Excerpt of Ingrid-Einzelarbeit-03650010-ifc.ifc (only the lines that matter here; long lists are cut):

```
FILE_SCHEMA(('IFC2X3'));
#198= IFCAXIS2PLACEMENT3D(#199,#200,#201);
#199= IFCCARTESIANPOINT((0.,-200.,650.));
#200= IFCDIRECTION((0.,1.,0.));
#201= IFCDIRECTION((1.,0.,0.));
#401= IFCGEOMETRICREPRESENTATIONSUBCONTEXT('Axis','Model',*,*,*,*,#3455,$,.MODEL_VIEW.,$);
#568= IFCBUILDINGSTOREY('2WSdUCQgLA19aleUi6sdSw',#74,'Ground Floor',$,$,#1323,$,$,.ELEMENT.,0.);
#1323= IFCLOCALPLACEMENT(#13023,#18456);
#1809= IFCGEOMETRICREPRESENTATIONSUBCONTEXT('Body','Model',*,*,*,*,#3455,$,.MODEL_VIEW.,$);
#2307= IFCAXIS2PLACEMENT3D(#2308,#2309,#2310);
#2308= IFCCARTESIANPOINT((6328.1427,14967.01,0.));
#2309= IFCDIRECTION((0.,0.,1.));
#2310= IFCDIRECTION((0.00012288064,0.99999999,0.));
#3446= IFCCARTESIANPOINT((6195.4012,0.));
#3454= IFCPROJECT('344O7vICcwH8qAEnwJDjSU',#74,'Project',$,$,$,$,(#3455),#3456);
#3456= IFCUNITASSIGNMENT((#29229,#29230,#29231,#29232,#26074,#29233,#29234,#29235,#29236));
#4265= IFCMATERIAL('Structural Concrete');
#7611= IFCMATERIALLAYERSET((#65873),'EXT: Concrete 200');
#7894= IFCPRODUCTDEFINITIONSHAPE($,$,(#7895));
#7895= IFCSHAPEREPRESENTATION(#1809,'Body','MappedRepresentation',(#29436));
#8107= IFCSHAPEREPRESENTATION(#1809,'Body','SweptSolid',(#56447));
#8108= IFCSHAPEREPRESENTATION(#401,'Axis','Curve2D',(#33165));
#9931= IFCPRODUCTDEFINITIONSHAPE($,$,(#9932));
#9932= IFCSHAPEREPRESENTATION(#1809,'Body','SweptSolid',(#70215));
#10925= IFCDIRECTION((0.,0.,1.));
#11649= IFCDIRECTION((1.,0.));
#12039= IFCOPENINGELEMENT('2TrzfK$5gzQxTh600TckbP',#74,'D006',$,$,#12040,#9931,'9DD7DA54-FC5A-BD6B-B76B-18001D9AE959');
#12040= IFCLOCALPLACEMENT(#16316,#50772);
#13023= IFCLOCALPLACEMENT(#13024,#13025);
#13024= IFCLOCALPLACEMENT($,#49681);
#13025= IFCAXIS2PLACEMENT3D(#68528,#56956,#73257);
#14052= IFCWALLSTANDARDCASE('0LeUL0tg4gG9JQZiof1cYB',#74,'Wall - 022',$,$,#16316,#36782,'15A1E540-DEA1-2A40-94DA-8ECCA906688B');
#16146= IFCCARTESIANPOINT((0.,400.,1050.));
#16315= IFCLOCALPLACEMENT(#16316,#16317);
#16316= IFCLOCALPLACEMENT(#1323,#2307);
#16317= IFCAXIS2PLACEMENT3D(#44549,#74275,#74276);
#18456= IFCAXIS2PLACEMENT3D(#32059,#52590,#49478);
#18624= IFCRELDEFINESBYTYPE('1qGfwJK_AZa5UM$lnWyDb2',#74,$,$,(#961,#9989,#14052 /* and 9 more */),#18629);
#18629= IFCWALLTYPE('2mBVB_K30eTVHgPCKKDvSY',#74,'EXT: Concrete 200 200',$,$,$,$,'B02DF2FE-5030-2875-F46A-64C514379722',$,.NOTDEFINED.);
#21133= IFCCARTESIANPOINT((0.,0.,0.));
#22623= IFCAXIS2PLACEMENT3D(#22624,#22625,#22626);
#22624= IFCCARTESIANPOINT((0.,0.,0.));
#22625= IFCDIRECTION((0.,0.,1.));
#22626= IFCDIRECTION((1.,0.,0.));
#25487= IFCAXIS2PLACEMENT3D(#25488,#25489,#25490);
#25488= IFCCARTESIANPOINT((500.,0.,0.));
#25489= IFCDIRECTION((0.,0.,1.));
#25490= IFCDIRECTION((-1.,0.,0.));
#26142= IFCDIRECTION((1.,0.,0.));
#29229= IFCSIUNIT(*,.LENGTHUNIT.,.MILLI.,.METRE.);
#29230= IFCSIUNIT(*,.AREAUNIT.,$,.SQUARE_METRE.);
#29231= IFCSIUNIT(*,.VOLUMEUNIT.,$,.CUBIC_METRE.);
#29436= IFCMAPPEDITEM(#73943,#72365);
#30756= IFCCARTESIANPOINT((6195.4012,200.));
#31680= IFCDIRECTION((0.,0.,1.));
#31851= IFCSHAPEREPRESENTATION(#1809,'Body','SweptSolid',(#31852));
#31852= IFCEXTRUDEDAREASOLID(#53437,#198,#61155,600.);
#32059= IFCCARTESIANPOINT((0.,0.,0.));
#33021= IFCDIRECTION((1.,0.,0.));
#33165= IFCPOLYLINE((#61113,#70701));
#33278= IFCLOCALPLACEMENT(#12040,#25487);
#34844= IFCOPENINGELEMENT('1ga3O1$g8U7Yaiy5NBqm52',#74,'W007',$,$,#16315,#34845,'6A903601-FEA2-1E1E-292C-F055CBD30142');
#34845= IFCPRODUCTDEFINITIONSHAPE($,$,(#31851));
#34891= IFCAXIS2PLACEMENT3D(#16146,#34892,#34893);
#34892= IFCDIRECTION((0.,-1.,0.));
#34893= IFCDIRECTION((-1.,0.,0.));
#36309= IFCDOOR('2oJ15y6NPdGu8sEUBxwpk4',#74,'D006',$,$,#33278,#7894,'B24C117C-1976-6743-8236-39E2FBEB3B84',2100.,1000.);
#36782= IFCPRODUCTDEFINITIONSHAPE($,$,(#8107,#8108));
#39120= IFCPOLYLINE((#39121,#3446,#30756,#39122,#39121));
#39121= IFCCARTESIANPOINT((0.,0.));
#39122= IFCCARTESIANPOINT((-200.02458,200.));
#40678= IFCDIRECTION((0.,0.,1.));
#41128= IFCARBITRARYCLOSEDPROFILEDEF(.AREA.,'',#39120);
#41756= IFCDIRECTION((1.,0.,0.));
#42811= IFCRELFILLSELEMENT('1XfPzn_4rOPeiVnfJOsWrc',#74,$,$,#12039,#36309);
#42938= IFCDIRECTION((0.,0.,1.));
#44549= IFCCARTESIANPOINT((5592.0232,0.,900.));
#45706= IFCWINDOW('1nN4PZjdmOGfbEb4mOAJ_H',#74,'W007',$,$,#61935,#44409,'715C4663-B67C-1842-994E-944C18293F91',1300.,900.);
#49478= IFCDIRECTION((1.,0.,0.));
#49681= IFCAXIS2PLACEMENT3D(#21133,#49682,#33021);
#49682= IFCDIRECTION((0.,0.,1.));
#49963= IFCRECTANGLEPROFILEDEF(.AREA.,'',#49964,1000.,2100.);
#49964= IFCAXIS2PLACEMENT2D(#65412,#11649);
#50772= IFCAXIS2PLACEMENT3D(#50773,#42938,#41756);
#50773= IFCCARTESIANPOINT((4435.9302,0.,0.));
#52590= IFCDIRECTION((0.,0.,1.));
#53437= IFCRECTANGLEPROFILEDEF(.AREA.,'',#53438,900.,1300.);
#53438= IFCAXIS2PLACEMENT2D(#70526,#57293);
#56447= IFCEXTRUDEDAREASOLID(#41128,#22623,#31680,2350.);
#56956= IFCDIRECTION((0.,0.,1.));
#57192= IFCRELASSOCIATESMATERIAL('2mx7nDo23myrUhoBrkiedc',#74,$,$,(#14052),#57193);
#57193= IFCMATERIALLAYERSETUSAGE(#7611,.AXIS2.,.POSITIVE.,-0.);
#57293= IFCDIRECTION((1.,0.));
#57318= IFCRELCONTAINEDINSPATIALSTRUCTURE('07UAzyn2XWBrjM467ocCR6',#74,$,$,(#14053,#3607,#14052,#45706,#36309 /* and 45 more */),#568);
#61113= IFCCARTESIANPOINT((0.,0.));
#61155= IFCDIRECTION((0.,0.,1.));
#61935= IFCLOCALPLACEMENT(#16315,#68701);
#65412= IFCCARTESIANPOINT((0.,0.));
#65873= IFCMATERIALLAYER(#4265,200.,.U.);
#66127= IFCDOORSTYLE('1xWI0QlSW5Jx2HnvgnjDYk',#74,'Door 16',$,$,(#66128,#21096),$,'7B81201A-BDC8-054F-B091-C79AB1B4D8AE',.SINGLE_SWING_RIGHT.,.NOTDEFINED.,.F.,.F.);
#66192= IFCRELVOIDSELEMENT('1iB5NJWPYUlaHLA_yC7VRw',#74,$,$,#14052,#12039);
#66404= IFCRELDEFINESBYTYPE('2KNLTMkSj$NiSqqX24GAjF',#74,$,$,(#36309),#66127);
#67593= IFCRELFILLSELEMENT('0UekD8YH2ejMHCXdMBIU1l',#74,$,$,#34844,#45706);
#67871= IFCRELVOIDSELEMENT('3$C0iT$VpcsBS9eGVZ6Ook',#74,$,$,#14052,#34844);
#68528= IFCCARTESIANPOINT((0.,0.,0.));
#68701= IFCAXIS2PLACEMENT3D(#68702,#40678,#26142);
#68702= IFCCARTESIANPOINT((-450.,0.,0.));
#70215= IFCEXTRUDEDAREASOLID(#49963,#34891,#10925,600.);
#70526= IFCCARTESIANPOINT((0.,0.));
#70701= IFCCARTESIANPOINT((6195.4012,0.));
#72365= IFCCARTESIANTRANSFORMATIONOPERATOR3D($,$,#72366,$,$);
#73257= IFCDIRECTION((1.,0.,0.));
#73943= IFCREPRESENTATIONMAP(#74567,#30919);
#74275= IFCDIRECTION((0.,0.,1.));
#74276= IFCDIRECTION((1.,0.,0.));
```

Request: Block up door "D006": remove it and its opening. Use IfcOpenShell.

```python
import ifcopenshell
import ifcopenshell.api.feature
import ifcopenshell.api.root
import ifcopenshell.geom
import ifcopenshell.util.shape

model = ifcopenshell.open("Ingrid-Einzelarbeit-03650010-ifc.ifc")
settings = ifcopenshell.geom.settings()


def volume(element):
    """Net volume in cubic metres, openings subtracted."""
    shape = ifcopenshell.geom.create_shape(settings, element)
    return ifcopenshell.util.shape.get_volume(shape.geometry)


door = model.by_guid("2oJ15y6NPdGu8sEUBxwpk4")
opening = door.FillsVoids[0].RelatingOpeningElement
wall = opening.VoidsElements[0].RelatingBuildingElement
before = volume(wall)

ifcopenshell.api.root.remove_product(model, product=door)
ifcopenshell.api.feature.remove_feature(model, feature=opening)

after = volume(wall)

print(f"wall volume {before:.3f} -> {after:.3f} m3")

model.write("Ingrid-Einzelarbeit-03650010-ifc_edited.ifc")
```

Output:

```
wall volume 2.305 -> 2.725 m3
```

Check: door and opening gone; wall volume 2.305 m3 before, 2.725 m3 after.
